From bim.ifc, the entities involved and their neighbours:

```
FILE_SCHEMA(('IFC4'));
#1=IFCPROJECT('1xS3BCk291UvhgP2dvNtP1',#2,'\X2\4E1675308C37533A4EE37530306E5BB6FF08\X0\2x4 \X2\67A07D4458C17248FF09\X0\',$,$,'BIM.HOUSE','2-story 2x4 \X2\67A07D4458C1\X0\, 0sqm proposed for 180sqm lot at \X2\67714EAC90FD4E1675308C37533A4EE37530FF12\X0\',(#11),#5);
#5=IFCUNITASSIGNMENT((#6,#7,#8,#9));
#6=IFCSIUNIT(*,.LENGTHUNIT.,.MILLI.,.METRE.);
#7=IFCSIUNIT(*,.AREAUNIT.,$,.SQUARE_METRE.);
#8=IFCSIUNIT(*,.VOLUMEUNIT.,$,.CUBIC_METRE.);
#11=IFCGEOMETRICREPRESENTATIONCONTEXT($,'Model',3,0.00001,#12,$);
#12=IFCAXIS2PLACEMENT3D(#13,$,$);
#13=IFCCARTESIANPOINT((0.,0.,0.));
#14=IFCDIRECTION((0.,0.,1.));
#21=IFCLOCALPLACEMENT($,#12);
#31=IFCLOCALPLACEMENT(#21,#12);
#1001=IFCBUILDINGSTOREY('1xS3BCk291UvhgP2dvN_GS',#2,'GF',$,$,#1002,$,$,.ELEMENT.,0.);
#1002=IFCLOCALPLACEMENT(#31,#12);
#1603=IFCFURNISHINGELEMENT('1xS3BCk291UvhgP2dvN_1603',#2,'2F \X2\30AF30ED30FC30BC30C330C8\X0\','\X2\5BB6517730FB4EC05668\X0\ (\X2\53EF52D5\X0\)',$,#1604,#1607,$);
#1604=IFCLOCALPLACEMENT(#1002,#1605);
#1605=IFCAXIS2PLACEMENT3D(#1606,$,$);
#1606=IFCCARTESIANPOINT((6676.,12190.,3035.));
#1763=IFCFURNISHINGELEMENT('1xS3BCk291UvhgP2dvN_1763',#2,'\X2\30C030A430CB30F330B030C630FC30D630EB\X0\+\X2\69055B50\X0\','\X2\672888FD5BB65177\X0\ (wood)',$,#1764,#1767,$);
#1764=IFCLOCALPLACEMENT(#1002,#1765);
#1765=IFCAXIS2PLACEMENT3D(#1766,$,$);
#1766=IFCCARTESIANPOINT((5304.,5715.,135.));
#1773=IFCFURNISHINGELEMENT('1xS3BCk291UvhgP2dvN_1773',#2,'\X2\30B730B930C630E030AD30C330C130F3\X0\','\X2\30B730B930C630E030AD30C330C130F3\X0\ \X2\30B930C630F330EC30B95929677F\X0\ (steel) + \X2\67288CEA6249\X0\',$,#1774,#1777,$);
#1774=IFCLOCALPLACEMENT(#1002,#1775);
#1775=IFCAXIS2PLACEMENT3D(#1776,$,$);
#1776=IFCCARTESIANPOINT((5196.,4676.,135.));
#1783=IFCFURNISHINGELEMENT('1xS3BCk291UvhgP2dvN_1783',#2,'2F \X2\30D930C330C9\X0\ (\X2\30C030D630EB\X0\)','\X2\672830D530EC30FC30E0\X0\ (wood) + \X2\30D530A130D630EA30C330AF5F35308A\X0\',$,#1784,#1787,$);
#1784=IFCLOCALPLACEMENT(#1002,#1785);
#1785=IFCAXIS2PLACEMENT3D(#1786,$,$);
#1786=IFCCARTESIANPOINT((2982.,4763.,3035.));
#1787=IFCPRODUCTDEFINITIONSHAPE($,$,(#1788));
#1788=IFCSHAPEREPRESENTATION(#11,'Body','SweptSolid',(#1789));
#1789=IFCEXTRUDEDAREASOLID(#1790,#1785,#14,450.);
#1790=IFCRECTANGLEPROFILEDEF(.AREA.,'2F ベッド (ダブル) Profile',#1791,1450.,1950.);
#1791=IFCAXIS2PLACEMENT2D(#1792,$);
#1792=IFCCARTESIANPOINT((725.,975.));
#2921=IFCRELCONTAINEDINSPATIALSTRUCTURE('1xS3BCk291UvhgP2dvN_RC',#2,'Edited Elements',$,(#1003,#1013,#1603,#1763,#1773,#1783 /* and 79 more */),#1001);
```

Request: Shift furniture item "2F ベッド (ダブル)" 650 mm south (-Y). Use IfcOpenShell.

```python
import ifcopenshell
import ifcopenshell.api.geometry
import ifcopenshell.util.placement

model = ifcopenshell.open("bim.ifc")

item = model.by_guid("1xS3BCk291UvhgP2dvN_1783")
matrix = ifcopenshell.util.placement.get_local_placement(item.ObjectPlacement)
matrix[1, 3] -= 650.0
ifcopenshell.api.geometry.edit_object_placement(model, product=item, matrix=matrix, is_si=False)

print(ifcopenshell.util.placement.get_local_placement(item.ObjectPlacement).round(3) + 0.0)

model.write("bim-out.ifc")
```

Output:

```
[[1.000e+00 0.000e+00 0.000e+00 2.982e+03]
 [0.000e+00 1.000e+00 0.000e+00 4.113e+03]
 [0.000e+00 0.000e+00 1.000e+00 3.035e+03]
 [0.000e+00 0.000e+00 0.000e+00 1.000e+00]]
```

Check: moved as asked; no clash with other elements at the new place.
